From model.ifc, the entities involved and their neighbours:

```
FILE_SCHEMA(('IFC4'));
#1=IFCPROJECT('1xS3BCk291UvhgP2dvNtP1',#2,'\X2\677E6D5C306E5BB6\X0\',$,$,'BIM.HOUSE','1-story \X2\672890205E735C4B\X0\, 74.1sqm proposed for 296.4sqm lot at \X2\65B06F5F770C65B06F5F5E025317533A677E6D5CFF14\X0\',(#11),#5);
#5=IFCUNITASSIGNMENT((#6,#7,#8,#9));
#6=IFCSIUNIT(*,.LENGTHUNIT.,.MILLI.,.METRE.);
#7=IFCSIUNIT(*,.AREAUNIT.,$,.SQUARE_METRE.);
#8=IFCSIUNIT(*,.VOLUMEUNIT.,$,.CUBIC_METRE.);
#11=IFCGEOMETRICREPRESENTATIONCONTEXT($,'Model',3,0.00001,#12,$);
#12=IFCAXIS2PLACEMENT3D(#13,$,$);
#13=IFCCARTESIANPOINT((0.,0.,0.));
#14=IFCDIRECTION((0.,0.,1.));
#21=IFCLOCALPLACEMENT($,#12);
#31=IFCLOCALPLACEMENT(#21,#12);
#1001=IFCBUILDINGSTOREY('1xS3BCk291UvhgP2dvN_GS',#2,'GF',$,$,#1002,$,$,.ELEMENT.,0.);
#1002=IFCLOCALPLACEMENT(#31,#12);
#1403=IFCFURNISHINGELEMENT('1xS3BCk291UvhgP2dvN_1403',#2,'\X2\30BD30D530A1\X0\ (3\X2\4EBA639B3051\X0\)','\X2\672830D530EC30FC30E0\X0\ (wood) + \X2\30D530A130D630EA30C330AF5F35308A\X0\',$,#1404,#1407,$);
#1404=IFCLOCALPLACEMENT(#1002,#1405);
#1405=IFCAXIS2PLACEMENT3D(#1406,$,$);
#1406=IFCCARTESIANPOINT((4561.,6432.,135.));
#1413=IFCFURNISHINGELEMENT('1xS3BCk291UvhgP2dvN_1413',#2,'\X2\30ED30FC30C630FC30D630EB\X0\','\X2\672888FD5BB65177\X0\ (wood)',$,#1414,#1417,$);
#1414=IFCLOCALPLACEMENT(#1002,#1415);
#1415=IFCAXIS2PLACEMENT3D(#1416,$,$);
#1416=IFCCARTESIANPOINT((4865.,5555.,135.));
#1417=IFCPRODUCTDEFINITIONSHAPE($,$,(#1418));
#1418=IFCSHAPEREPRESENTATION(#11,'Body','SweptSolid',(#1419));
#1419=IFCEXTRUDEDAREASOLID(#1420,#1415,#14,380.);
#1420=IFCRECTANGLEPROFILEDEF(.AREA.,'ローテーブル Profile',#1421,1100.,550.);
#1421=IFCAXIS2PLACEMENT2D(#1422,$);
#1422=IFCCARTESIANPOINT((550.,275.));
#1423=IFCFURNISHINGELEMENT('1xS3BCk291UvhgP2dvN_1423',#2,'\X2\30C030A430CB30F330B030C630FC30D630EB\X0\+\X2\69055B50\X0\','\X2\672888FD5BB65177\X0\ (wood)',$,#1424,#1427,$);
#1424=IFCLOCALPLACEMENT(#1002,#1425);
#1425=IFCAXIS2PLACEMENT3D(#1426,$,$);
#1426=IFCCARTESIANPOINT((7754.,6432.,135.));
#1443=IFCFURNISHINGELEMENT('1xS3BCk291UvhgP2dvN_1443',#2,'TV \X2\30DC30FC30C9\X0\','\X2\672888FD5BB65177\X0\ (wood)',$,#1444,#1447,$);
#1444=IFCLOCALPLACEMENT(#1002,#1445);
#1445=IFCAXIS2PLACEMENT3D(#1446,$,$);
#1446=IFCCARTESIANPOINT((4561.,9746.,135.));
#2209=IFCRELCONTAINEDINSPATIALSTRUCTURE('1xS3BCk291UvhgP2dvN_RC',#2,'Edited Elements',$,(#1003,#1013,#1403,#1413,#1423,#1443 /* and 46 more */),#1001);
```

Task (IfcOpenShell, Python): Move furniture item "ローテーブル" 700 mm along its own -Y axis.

```python
import ifcopenshell
import ifcopenshell.api.geometry
import ifcopenshell.util.placement

model = ifcopenshell.open("model.ifc")

item = model.by_guid("1xS3BCk291UvhgP2dvN_1413")
matrix = ifcopenshell.util.placement.get_local_placement(item.ObjectPlacement)
matrix[:3, 3] -= matrix[:3, 1] * 700.0
ifcopenshell.api.geometry.edit_object_placement(model, product=item, matrix=matrix, is_si=False)

print(ifcopenshell.util.placement.get_local_placement(item.ObjectPlacement).round(3) + 0.0)

model.write("model_rev.ifc")
```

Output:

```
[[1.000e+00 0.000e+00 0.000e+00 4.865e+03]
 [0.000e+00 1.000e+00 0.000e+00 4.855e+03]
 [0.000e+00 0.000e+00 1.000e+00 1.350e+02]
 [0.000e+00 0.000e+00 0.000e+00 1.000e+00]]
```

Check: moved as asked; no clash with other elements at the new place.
